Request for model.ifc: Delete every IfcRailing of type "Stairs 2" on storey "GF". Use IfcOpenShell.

First a look at what the model holds.

```python
import ifcopenshell
import ifcopenshell.util.element

model = ifcopenshell.open("model.ifc")
print(model.schema)
storey = next(s for s in model.by_type("IfcBuildingStorey") if s.Name == "GF")
railings = [e for e in ifcopenshell.util.element.get_decomposition(storey) if e.is_a("IfcRailing")]
seen = {}
for e in railings:
    element_type = ifcopenshell.util.element.get_type(e)
    name = element_type.Name if element_type not in (None, e) else None
    seen[name] = seen.get(name, 0) + 1
for name, count in sorted(seen.items(), key=str):
    print(count, "x", name)
```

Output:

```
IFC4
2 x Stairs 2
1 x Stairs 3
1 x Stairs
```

```python
import ifcopenshell
import ifcopenshell.api.root
import ifcopenshell.util.element

model = ifcopenshell.open("model.ifc")

storey = next(s for s in model.by_type("IfcBuildingStorey") if s.Name == "GF")
railings = [e for e in ifcopenshell.util.element.get_decomposition(storey) if e.is_a("IfcRailing")]
targets = [e for e in railings if (t := ifcopenshell.util.element.get_type(e)) not in (None, e) and t.Name == "Stairs 2"]

for e in targets:
    ifcopenshell.api.root.remove_product(model, product=e)
print(len(targets), "removed")

model.write("model_v2.ifc")
```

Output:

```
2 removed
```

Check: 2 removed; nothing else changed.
